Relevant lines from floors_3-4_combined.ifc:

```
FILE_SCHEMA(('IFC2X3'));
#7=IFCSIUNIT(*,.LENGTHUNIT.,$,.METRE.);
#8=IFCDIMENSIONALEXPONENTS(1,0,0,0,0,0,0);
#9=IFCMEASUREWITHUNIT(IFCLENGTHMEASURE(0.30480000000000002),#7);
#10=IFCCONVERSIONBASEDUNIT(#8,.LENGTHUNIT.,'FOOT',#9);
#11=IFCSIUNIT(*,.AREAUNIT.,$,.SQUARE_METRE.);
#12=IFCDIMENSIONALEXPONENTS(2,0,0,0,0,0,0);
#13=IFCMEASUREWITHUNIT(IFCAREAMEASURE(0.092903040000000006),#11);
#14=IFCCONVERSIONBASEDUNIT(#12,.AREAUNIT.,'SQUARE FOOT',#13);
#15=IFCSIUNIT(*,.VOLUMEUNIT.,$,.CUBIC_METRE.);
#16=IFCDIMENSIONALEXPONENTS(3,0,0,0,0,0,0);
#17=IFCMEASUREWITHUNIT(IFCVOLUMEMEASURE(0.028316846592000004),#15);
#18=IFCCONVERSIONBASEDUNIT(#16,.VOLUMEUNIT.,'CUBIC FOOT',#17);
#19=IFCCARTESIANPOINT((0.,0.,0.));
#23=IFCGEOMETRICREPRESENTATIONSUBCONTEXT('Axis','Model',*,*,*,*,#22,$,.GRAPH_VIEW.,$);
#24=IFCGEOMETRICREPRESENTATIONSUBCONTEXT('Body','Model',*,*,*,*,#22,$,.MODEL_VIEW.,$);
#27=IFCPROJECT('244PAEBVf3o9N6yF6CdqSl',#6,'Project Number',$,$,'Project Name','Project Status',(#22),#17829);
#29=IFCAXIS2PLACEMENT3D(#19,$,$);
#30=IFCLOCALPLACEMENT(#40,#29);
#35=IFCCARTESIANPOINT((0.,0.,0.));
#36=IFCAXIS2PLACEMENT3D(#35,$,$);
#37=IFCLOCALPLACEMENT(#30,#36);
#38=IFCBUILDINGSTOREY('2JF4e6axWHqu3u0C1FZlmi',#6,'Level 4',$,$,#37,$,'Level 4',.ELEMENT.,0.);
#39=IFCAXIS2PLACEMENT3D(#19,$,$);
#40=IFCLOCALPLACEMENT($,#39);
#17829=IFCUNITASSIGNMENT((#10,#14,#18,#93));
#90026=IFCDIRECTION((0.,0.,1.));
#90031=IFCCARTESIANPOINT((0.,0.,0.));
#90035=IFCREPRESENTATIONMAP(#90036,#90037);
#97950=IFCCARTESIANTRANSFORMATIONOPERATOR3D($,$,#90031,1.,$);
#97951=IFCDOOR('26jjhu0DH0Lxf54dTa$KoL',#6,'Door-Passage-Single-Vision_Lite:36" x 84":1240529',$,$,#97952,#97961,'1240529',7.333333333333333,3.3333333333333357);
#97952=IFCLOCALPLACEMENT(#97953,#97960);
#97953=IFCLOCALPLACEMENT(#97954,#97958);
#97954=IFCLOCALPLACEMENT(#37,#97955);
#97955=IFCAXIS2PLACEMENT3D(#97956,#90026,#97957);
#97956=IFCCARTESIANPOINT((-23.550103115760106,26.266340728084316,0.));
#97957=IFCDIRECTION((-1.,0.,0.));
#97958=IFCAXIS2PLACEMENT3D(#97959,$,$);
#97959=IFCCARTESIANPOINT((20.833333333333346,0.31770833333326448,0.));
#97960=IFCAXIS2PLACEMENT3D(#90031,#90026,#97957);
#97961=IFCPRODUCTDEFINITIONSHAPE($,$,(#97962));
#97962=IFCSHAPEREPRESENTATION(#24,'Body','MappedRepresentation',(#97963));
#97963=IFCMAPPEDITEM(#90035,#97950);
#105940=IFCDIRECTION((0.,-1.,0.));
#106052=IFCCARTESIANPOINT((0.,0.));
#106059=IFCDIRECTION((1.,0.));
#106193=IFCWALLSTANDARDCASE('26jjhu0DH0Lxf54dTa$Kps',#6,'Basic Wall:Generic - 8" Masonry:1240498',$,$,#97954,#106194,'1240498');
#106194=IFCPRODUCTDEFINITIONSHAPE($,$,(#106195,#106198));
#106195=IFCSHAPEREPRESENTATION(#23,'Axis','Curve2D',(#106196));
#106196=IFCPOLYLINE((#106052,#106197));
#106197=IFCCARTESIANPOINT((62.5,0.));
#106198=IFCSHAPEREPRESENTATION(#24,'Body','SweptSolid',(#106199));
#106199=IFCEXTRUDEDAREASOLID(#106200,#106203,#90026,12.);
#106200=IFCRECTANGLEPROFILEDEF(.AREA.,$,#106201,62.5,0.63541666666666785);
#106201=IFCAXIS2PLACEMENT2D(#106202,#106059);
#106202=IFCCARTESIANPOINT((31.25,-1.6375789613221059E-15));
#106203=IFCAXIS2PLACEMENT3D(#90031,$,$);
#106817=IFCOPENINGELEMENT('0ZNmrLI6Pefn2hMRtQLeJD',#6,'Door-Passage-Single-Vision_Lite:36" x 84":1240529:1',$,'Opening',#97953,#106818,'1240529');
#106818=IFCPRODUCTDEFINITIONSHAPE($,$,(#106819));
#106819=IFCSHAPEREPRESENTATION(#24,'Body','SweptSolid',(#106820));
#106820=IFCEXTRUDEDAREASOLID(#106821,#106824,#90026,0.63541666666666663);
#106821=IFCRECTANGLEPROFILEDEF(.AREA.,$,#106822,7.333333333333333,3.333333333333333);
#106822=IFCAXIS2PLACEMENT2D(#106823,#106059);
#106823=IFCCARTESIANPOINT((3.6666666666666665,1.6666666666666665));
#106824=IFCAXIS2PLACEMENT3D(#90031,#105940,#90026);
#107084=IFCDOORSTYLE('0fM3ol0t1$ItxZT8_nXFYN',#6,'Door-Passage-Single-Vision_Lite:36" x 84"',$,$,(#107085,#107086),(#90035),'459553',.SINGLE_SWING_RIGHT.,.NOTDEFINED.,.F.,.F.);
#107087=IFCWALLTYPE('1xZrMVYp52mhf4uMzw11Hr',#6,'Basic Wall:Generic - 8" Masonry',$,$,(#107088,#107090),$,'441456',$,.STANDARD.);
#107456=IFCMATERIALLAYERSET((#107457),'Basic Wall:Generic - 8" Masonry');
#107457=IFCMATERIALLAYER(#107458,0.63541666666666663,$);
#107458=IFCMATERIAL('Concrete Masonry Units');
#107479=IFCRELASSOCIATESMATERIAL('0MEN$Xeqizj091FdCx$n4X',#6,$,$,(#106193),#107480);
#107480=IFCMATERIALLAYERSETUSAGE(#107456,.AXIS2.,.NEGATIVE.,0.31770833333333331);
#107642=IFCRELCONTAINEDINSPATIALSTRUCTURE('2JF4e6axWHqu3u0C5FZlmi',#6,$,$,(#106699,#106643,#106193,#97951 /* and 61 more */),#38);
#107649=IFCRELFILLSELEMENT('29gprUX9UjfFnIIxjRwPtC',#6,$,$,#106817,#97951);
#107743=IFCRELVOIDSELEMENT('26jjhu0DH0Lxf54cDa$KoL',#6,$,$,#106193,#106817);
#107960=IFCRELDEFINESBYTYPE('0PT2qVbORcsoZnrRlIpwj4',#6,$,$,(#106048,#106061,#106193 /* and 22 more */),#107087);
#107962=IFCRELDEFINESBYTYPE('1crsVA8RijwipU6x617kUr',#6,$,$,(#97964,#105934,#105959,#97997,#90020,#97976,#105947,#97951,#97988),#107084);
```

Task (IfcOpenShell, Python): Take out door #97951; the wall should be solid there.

```python
import ifcopenshell
import ifcopenshell.api.feature
import ifcopenshell.api.root
import ifcopenshell.geom
import ifcopenshell.util.shape

model = ifcopenshell.open("floors_3-4_combined.ifc")
settings = ifcopenshell.geom.settings()


def volume(element):
    """Net volume in cubic metres, openings subtracted."""
    shape = ifcopenshell.geom.create_shape(settings, element)
    return ifcopenshell.util.shape.get_volume(shape.geometry)


door = model.by_id(97951)
opening = door.FillsVoids[0].RelatingOpeningElement
wall = opening.VoidsElements[0].RelatingBuildingElement
before = volume(wall)

ifcopenshell.api.root.remove_product(model, product=door)
ifcopenshell.api.feature.remove_feature(model, feature=opening)

after = volume(wall)

print(f"wall volume {before:.3f} -> {after:.3f} m3")

model.write("floors_3-4_combined_rev.ifc")
```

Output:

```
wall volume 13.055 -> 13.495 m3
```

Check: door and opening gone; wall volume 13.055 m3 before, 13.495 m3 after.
